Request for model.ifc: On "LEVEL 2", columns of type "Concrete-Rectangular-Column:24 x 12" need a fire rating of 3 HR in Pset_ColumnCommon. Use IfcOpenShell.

First a look at what the model holds.

```python
import ifcopenshell
import ifcopenshell.util.element

model = ifcopenshell.open("model.ifc")
print(model.schema)
storey = next(s for s in model.by_type("IfcBuildingStorey") if s.Name == "LEVEL 2")
columns = [e for e in ifcopenshell.util.element.get_decomposition(storey) if e.is_a("IfcColumn")]
seen = {}
for e in columns:
    element_type = ifcopenshell.util.element.get_type(e)
    key = (element_type.Name if element_type != e and element_type else None, ifcopenshell.util.element.get_pset(e, "Pset_ColumnCommon", "FireRating"))
    seen[key] = seen.get(key, 0) + 1
for (name, value), count in sorted(seen.items(), key=str):
    print(count, "x", name, "|", value)
```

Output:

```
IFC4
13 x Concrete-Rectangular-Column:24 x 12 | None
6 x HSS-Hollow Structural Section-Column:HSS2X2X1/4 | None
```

```python
import ifcopenshell
import ifcopenshell.api.pset
import ifcopenshell.util.element

model = ifcopenshell.open("model.ifc")

storey = next(s for s in model.by_type("IfcBuildingStorey") if s.Name == "LEVEL 2")
columns = [e for e in ifcopenshell.util.element.get_decomposition(storey) if e.is_a("IfcColumn")]

count = 0
for e in columns:
    element_type = ifcopenshell.util.element.get_type(e)
    if element_type in (None, e) or element_type.Name != "Concrete-Rectangular-Column:24 x 12":
        continue
    # add_pset returns the element's existing set when there is one.
    pset = ifcopenshell.api.pset.add_pset(model, product=e, name="Pset_ColumnCommon")
    ifcopenshell.api.pset.edit_pset(model, pset=pset, properties={"FireRating": "3 HR"})
    count += 1

print(count, "columns updated")

model.write("model_rev.ifc")
```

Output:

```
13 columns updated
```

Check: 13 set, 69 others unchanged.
